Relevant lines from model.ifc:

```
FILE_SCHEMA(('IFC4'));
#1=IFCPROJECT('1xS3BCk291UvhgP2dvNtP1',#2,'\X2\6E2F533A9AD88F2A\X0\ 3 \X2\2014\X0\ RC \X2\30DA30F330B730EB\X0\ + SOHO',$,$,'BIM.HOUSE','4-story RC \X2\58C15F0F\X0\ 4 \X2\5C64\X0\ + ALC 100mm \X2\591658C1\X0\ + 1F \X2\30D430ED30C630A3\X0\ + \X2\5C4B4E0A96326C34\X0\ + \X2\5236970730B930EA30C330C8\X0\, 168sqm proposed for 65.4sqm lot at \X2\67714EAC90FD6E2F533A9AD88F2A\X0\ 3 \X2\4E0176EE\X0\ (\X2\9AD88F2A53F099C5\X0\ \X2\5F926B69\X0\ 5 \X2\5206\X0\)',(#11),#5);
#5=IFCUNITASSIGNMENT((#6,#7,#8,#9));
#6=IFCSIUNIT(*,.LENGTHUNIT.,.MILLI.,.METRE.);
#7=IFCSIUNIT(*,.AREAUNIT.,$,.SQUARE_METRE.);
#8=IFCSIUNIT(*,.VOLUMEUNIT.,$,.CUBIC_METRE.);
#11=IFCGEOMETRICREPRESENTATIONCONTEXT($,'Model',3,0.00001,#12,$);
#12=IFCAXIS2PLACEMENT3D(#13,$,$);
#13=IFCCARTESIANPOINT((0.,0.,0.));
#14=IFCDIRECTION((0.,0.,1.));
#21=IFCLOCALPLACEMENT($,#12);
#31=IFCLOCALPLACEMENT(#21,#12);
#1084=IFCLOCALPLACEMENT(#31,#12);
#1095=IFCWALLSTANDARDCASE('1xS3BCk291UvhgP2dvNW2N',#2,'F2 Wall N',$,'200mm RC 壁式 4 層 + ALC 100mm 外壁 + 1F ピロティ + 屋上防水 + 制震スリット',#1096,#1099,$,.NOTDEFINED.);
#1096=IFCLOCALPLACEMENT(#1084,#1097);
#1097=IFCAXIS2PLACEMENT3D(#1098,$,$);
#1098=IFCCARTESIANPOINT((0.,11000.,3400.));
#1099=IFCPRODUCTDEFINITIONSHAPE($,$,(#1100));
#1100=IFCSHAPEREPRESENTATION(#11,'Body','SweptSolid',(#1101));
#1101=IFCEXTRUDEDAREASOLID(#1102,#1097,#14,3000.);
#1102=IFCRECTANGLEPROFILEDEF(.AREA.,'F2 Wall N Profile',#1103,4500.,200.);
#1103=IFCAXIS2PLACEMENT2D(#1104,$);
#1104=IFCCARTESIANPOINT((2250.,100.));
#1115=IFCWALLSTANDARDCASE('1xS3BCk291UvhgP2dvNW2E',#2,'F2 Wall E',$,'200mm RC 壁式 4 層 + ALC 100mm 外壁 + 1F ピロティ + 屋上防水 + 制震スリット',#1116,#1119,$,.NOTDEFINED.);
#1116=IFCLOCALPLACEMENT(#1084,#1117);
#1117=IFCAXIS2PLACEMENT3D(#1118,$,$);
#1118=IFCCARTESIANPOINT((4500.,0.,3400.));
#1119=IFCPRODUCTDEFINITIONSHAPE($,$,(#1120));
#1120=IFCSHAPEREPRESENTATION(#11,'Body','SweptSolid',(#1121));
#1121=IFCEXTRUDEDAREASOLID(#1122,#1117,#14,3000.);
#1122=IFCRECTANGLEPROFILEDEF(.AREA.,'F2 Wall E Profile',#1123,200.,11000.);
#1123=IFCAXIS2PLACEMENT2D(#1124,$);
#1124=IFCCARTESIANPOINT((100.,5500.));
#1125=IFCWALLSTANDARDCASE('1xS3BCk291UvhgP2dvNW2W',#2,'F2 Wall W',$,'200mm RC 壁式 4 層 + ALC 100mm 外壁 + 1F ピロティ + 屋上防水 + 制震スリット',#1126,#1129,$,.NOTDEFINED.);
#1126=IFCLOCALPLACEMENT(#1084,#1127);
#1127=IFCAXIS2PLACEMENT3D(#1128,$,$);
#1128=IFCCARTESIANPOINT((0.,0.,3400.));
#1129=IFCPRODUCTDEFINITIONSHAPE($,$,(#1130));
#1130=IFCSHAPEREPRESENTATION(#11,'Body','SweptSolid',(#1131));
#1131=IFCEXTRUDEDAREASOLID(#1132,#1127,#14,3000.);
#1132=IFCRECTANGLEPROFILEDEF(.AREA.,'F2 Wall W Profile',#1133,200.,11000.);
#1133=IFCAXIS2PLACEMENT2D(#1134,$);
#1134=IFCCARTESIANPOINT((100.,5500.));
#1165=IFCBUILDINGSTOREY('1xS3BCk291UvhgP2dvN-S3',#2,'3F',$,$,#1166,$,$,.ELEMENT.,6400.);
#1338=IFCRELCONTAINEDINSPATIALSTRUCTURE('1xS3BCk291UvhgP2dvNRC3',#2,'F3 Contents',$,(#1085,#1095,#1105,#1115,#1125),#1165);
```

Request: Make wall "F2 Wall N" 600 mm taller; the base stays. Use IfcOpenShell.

```python
import ifcopenshell
import ifcopenshell.geom
import ifcopenshell.util.shape
import ifcopenshell.util.unit

model = ifcopenshell.open("model.ifc")
unit_scale = ifcopenshell.util.unit.calculate_unit_scale(model)
settings = ifcopenshell.geom.settings()


def volume(element):
    """Net volume in cubic metres, openings subtracted."""
    shape = ifcopenshell.geom.create_shape(settings, element)
    return ifcopenshell.util.shape.get_volume(shape.geometry)


wall = model.by_id(1095)
before = volume(wall)

body = next(r for r in wall.Representation.Representations if r.RepresentationIdentifier == "Body")
solid = body.Items[0]
old_height = solid.Depth
solid.Depth += 0.6 / unit_scale
after = volume(wall)

print(f"height {old_height:g} -> {solid.Depth:g}, volume {before:.3f} -> {after:.3f} m3")

model.write("model_edited.ifc")
```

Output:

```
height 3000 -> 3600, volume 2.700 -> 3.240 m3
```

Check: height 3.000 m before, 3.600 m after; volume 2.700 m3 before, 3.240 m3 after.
